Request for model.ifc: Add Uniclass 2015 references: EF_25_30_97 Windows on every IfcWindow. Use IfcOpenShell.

First a look at what the model holds.

```python
import ifcopenshell

model = ifcopenshell.open("model.ifc")
print(model.schema)
print("classifications:", [c.Name for c in model.by_type("IfcClassification")])
for ifc_class in ("IfcDoor", "IfcRoof", "IfcStair", "IfcWall", "IfcWindow"):
    print(ifc_class, len(model.by_type(ifc_class)))
```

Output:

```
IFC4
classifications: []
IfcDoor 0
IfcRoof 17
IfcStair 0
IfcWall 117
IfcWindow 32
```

```python
import ifcopenshell
import ifcopenshell.api.classification

model = ifcopenshell.open("model.ifc")

system = ifcopenshell.api.classification.add_classification(model, classification="Uniclass 2015")

codes = {
    "IfcWindow": ("EF_25_30_97", "Windows"),
}
for ifc_class, (code, name) in codes.items():
    products = model.by_type(ifc_class)
    ifcopenshell.api.classification.add_reference(
        model, products=products, classification=system, identification=code, name=name
    )
    print(code, len(products))

model.write("model_rev.ifc")
```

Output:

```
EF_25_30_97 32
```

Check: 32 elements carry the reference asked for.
